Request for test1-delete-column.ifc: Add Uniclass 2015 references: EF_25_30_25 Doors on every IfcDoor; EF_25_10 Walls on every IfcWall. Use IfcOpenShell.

First a look at what the model holds.

```python
import ifcopenshell

model = ifcopenshell.open("test1-delete-column.ifc")
print(model.schema)
print("classifications:", [c.Name for c in model.by_type("IfcClassification")])
for ifc_class in ("IfcDoor", "IfcRoof", "IfcStair", "IfcWall", "IfcWindow"):
    print(ifc_class, len(model.by_type(ifc_class)))
```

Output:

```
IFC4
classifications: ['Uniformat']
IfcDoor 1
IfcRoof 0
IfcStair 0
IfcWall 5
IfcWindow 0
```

```python
import ifcopenshell
import ifcopenshell.api.classification

model = ifcopenshell.open("test1-delete-column.ifc")

system = ifcopenshell.api.classification.add_classification(model, classification="Uniclass 2015")

codes = {
    "IfcDoor": ("EF_25_30_25", "Doors"),
    "IfcWall": ("EF_25_10", "Walls"),
}
for ifc_class, (code, name) in codes.items():
    products = model.by_type(ifc_class)
    ifcopenshell.api.classification.add_reference(
        model, products=products, classification=system, identification=code, name=name
    )
    print(code, len(products))

model.write("test1-delete-column_v2.ifc")
```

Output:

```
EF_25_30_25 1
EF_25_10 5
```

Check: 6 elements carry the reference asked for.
